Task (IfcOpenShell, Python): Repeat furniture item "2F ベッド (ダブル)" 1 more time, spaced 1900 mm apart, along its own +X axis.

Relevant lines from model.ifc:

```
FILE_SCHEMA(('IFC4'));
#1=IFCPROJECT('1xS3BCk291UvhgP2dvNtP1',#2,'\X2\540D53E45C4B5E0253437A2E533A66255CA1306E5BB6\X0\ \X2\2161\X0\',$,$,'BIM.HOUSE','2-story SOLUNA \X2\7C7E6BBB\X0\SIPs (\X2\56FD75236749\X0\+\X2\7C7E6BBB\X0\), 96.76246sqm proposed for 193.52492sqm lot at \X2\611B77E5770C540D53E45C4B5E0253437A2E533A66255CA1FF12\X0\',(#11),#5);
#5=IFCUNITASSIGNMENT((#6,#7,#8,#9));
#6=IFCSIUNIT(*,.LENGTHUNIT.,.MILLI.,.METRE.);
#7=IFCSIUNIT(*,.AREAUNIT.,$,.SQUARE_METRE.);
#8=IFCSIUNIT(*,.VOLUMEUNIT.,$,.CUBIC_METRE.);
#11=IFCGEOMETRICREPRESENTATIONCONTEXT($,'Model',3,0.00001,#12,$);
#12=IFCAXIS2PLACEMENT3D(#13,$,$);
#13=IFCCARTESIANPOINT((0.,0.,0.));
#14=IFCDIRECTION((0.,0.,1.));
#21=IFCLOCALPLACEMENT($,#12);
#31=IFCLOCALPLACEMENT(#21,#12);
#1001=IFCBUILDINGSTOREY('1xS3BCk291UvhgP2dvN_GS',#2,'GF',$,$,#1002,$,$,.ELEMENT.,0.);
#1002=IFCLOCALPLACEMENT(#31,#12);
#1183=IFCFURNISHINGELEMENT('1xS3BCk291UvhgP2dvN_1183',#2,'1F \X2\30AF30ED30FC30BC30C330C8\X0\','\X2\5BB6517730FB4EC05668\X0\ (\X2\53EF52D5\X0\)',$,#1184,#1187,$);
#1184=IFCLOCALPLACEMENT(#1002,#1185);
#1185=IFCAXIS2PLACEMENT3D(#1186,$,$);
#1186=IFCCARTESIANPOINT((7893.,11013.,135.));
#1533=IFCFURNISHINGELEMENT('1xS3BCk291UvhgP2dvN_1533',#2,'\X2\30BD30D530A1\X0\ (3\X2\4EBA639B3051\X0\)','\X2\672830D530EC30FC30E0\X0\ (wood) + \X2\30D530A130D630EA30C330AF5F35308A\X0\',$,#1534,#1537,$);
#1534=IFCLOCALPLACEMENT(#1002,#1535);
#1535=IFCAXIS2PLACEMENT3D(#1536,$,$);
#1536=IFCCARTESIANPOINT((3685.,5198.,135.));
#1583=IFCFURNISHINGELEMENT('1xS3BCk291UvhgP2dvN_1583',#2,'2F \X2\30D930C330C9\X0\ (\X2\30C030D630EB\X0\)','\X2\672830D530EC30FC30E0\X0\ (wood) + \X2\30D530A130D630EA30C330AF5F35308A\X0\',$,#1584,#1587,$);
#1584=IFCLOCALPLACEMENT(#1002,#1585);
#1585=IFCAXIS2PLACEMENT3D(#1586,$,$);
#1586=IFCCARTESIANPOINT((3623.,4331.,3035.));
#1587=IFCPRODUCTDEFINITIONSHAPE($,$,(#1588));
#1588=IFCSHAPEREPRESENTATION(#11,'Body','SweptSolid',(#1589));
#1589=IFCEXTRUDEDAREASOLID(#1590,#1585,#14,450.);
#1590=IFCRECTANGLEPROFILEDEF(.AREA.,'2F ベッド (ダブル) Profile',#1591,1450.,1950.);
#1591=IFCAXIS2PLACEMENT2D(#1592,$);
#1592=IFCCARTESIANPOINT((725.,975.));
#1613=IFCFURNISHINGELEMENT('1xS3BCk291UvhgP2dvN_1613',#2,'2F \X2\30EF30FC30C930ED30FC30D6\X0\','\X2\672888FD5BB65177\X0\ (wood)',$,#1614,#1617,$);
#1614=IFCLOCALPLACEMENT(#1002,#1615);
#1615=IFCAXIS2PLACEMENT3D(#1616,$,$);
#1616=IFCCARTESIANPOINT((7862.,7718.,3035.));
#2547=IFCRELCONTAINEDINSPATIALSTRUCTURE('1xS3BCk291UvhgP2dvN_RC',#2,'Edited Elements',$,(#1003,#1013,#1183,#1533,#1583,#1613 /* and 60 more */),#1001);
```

```python
import ifcopenshell
import ifcopenshell.api.geometry
import ifcopenshell.api.root
import ifcopenshell.util.element
import ifcopenshell.util.placement

model = ifcopenshell.open("model.ifc")


def reuse_history(source, copy):
    """copy_class also copies each property set's owner history, people and application; keep the originals."""
    for rel in copy.IsDefinedBy:
        if rel.is_a("IfcRelDefinesByProperties") and (history := rel.RelatingPropertyDefinition.OwnerHistory):
            rel.RelatingPropertyDefinition.OwnerHistory = source.OwnerHistory
            ifcopenshell.util.element.remove_deep2(model, history)


source = model.by_guid("1xS3BCk291UvhgP2dvN_1583")
base = ifcopenshell.util.placement.get_local_placement(source.ObjectPlacement)
step = base[:3, 0] * 1900.0

for i in range(1, 2):
    copy = ifcopenshell.api.root.copy_class(model, product=source)
    copy.Representation = ifcopenshell.util.element.copy_deep(
        model, source.Representation, exclude=["IfcGeometricRepresentationContext", "IfcRepresentationMap"]
    )
    reuse_history(source, copy)
    matrix = base.copy()
    matrix[:3, 3] += i * step
    print("added at", matrix[:3, 3].round(3) + 0.0)
    ifcopenshell.api.geometry.edit_object_placement(model, product=copy, matrix=matrix, is_si=False)

model.write("model_updated.ifc")
```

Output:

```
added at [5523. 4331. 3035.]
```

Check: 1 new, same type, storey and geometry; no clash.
